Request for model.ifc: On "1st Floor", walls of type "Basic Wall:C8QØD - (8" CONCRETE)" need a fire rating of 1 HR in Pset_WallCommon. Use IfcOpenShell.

First a look at what the model holds.

```python
import ifcopenshell
import ifcopenshell.util.element

model = ifcopenshell.open("model.ifc")
print(model.schema)
storey = next(s for s in model.by_type("IfcBuildingStorey") if s.Name == "1st Floor")
walls = [e for e in ifcopenshell.util.element.get_decomposition(storey) if e.is_a("IfcWall")]
seen = {}
for e in walls:
    element_type = ifcopenshell.util.element.get_type(e)
    key = (element_type.Name if element_type != e and element_type else None, ifcopenshell.util.element.get_pset(e, "Pset_WallCommon", "FireRating"))
    seen[key] = seen.get(key, 0) + 1
for (name, value), count in sorted(seen.items(), key=str):
    print(count, "x", name, "|", value)
```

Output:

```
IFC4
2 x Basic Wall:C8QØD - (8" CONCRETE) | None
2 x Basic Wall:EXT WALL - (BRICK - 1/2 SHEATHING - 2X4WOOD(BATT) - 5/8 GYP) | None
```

```python
import ifcopenshell
import ifcopenshell.api.pset
import ifcopenshell.util.element

model = ifcopenshell.open("model.ifc")

storey = next(s for s in model.by_type("IfcBuildingStorey") if s.Name == "1st Floor")
walls = [e for e in ifcopenshell.util.element.get_decomposition(storey) if e.is_a("IfcWall")]

count = 0
for e in walls:
    element_type = ifcopenshell.util.element.get_type(e)
    if element_type in (None, e) or element_type.Name != 'Basic Wall:C8QØD - (8" CONCRETE)':
        continue
    # add_pset returns the element's existing set when there is one.
    pset = ifcopenshell.api.pset.add_pset(model, product=e, name="Pset_WallCommon")
    ifcopenshell.api.pset.edit_pset(model, pset=pset, properties={"FireRating": "1 HR"})
    count += 1

print(count, "walls updated")

model.write("model_updated.ifc")
```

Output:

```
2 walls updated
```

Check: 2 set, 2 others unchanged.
